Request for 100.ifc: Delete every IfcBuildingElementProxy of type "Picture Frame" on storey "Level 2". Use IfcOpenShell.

First a look at what the model holds.

```python
import ifcopenshell
import ifcopenshell.util.element

model = ifcopenshell.open("100.ifc")
print(model.schema)
storey = next(s for s in model.by_type("IfcBuildingStorey") if s.Name == "Level 2")
proxies = [e for e in ifcopenshell.util.element.get_decomposition(storey) if e.is_a("IfcBuildingElementProxy")]
seen = {}
for e in proxies:
    element_type = ifcopenshell.util.element.get_type(e)
    name = element_type.Name if element_type not in (None, e) else None
    seen[name] = seen.get(name, 0) + 1
for name, count in sorted(seen.items(), key=str):
    print(count, "x", name)
```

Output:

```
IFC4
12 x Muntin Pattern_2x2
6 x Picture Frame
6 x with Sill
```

```python
import ifcopenshell
import ifcopenshell.api.root
import ifcopenshell.util.element

model = ifcopenshell.open("100.ifc")

storey = next(s for s in model.by_type("IfcBuildingStorey") if s.Name == "Level 2")
proxies = [e for e in ifcopenshell.util.element.get_decomposition(storey) if e.is_a("IfcBuildingElementProxy")]
targets = [e for e in proxies if (t := ifcopenshell.util.element.get_type(e)) not in (None, e) and t.Name == "Picture Frame"]

for e in targets:
    ifcopenshell.api.root.remove_product(model, product=e)
print(len(targets), "removed")

model.write("100_edited.ifc")
```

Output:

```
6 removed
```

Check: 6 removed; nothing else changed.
